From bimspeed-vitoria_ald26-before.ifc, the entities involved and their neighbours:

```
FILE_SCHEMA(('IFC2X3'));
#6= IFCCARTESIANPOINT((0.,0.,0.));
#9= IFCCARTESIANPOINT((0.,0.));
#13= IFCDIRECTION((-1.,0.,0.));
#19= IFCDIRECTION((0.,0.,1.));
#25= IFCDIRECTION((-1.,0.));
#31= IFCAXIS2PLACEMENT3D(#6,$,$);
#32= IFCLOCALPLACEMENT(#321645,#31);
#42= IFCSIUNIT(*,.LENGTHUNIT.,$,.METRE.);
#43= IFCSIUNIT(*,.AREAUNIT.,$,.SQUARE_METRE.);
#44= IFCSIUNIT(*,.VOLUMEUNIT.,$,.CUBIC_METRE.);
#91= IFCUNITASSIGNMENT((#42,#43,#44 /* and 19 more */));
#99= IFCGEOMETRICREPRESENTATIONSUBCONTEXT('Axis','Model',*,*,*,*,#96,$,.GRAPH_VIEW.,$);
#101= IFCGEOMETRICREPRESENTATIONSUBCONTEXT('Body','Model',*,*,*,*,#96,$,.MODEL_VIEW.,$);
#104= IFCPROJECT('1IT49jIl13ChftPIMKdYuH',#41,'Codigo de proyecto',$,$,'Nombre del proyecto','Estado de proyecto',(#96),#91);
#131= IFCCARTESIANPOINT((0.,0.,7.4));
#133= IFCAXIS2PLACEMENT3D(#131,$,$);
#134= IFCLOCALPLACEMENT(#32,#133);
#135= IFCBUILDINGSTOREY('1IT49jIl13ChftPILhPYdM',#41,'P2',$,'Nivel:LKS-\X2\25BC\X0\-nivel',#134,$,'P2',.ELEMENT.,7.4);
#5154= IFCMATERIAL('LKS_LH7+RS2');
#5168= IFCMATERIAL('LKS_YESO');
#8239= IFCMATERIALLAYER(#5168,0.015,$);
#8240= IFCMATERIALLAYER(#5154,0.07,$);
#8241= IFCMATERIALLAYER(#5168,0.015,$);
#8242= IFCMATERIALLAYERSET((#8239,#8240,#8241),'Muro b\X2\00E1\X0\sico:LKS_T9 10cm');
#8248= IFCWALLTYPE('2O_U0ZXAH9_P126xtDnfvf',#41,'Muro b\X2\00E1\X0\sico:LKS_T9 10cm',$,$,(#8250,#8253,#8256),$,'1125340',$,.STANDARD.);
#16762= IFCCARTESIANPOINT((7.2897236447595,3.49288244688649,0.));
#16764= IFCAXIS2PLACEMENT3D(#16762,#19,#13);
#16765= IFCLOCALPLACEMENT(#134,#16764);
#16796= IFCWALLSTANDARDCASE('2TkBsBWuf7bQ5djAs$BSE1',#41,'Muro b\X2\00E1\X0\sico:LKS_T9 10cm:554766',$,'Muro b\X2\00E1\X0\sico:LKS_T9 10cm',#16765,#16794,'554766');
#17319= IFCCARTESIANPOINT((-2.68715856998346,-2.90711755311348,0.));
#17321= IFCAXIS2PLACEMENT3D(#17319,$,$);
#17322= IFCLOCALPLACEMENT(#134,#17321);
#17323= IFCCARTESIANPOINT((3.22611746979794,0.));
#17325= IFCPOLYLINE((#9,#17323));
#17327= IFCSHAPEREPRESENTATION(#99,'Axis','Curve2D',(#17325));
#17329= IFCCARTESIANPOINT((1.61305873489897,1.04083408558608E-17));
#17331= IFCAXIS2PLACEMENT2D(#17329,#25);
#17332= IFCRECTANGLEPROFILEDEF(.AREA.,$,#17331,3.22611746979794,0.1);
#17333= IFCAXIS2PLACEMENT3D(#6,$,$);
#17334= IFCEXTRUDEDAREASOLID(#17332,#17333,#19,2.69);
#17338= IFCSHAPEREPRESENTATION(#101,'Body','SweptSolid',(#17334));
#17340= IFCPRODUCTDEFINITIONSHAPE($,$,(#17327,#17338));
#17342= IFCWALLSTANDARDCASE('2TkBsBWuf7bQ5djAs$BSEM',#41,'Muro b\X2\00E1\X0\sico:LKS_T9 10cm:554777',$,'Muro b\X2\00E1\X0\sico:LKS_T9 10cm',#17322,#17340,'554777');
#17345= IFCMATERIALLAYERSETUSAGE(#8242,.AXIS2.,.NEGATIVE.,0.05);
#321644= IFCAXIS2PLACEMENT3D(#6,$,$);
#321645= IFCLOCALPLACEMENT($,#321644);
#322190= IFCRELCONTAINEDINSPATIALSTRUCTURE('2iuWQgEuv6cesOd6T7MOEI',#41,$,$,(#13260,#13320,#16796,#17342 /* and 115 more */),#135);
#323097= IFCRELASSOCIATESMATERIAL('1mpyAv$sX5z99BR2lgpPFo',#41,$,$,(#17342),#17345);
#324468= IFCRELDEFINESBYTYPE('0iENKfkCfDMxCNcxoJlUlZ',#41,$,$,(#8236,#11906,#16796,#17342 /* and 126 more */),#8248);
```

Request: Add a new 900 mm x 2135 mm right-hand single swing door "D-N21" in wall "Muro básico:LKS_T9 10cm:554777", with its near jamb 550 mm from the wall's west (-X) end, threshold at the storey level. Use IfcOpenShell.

```python
import numpy as np
import ifcopenshell
import ifcopenshell.api.feature
import ifcopenshell.api.geometry
import ifcopenshell.api.root
import ifcopenshell.api.spatial
import ifcopenshell.api.type
import ifcopenshell.geom
import ifcopenshell.util.element
import ifcopenshell.util.placement
import ifcopenshell.util.representation
import ifcopenshell.util.shape
import ifcopenshell.util.unit

model = ifcopenshell.open("bimspeed-vitoria_ald26-before.ifc")
unit_scale = ifcopenshell.util.unit.calculate_unit_scale(model)
settings = ifcopenshell.geom.settings()


def volume(element):
    """Net volume in cubic metres, openings subtracted."""
    shape = ifcopenshell.geom.create_shape(settings, element)
    return ifcopenshell.util.shape.get_volume(shape.geometry)


wall = model.by_id(17342)
storey = ifcopenshell.util.element.get_container(wall, ifc_class="IfcBuildingStorey")
context = ifcopenshell.util.representation.get_context(model, "Model", "Body", "MODEL_VIEW")
before = volume(wall)

width, height, from_end, sill = 0.9, 2.135, 0.55, 0.0  # metres

# The wall runs along its own X axis, and the end named is its -X end.
wall_shape = ifcopenshell.geom.create_shape(settings, wall)
x, y, z = ifcopenshell.util.shape.get_vertices(wall_shape.geometry).T
start = x.min() + from_end
face, thickness = float(y.min()), float(y.max() - y.min())
wall_matrix = ifcopenshell.util.placement.get_local_placement(wall.ObjectPlacement)
level = ifcopenshell.util.placement.get_local_placement(storey.ObjectPlacement)[2, 3]


def in_wall(x, y):
    """Placement at x, y metres in the wall's axes, at sill height."""
    matrix = wall_matrix.copy()
    matrix[:, 3] = wall_matrix @ np.array([x / unit_scale, y / unit_scale, 0.0, 1.0])
    matrix[2, 3] = level + sill / unit_scale
    return matrix


# Opening: a box that overshoots both wall faces by 50 mm.
opening = ifcopenshell.api.root.create_entity(model, ifc_class="IfcOpeningElement")
box = ifcopenshell.api.geometry.add_wall_representation(
    model, context=context, length=width, height=height, thickness=thickness + 0.1
)
ifcopenshell.api.geometry.assign_representation(model, product=opening, representation=box)
ifcopenshell.api.geometry.edit_object_placement(model, product=opening, matrix=in_wall(start, face - 0.05), is_si=False)
ifcopenshell.api.feature.add_feature(model, feature=opening, element=wall)

door = ifcopenshell.api.root.create_entity(model, ifc_class="IfcDoor", name="D-N21")
door.OverallWidth, door.OverallHeight = width / unit_scale, height / unit_scale
body = ifcopenshell.api.geometry.add_door_representation(
    model,
    context=context,
    overall_width=door.OverallWidth,
    overall_height=door.OverallHeight,
    operation_type="SINGLE_SWING_RIGHT",
    lining_properties={"LiningDepth": thickness / unit_scale, "ThresholdDepth": thickness / unit_scale},
)
ifcopenshell.api.geometry.assign_representation(model, product=door, representation=body)
ifcopenshell.api.spatial.assign_container(model, products=[door], relating_structure=storey)
fills = ifcopenshell.api.feature.add_filling(model, opening=opening, element=door)
fills.OwnerHistory = door.OwnerHistory  # required in IFC2X3

# IFC2X3 keeps the operation on the door style.
style = ifcopenshell.api.root.create_entity(model, ifc_class="IfcDoorStyle", name="D-N21")
style.OperationType, style.ConstructionType = "SINGLE_SWING_RIGHT", "NOTDEFINED"
style.ParameterTakesPrecedence = style.Sizeable = False
ifcopenshell.api.type.assign_type(model, related_objects=[door], relating_type=style)

# The lining spans the wall, so the door starts at the wall face.
ifcopenshell.api.geometry.edit_object_placement(model, product=door, matrix=in_wall(start, face), is_si=False)

after = volume(wall)

print(f"wall volume {before:.3f} -> {after:.3f} m3")

model.write("bimspeed-vitoria_ald26-before_edited.ifc")
```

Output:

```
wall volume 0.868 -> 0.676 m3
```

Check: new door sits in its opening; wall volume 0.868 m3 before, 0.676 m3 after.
